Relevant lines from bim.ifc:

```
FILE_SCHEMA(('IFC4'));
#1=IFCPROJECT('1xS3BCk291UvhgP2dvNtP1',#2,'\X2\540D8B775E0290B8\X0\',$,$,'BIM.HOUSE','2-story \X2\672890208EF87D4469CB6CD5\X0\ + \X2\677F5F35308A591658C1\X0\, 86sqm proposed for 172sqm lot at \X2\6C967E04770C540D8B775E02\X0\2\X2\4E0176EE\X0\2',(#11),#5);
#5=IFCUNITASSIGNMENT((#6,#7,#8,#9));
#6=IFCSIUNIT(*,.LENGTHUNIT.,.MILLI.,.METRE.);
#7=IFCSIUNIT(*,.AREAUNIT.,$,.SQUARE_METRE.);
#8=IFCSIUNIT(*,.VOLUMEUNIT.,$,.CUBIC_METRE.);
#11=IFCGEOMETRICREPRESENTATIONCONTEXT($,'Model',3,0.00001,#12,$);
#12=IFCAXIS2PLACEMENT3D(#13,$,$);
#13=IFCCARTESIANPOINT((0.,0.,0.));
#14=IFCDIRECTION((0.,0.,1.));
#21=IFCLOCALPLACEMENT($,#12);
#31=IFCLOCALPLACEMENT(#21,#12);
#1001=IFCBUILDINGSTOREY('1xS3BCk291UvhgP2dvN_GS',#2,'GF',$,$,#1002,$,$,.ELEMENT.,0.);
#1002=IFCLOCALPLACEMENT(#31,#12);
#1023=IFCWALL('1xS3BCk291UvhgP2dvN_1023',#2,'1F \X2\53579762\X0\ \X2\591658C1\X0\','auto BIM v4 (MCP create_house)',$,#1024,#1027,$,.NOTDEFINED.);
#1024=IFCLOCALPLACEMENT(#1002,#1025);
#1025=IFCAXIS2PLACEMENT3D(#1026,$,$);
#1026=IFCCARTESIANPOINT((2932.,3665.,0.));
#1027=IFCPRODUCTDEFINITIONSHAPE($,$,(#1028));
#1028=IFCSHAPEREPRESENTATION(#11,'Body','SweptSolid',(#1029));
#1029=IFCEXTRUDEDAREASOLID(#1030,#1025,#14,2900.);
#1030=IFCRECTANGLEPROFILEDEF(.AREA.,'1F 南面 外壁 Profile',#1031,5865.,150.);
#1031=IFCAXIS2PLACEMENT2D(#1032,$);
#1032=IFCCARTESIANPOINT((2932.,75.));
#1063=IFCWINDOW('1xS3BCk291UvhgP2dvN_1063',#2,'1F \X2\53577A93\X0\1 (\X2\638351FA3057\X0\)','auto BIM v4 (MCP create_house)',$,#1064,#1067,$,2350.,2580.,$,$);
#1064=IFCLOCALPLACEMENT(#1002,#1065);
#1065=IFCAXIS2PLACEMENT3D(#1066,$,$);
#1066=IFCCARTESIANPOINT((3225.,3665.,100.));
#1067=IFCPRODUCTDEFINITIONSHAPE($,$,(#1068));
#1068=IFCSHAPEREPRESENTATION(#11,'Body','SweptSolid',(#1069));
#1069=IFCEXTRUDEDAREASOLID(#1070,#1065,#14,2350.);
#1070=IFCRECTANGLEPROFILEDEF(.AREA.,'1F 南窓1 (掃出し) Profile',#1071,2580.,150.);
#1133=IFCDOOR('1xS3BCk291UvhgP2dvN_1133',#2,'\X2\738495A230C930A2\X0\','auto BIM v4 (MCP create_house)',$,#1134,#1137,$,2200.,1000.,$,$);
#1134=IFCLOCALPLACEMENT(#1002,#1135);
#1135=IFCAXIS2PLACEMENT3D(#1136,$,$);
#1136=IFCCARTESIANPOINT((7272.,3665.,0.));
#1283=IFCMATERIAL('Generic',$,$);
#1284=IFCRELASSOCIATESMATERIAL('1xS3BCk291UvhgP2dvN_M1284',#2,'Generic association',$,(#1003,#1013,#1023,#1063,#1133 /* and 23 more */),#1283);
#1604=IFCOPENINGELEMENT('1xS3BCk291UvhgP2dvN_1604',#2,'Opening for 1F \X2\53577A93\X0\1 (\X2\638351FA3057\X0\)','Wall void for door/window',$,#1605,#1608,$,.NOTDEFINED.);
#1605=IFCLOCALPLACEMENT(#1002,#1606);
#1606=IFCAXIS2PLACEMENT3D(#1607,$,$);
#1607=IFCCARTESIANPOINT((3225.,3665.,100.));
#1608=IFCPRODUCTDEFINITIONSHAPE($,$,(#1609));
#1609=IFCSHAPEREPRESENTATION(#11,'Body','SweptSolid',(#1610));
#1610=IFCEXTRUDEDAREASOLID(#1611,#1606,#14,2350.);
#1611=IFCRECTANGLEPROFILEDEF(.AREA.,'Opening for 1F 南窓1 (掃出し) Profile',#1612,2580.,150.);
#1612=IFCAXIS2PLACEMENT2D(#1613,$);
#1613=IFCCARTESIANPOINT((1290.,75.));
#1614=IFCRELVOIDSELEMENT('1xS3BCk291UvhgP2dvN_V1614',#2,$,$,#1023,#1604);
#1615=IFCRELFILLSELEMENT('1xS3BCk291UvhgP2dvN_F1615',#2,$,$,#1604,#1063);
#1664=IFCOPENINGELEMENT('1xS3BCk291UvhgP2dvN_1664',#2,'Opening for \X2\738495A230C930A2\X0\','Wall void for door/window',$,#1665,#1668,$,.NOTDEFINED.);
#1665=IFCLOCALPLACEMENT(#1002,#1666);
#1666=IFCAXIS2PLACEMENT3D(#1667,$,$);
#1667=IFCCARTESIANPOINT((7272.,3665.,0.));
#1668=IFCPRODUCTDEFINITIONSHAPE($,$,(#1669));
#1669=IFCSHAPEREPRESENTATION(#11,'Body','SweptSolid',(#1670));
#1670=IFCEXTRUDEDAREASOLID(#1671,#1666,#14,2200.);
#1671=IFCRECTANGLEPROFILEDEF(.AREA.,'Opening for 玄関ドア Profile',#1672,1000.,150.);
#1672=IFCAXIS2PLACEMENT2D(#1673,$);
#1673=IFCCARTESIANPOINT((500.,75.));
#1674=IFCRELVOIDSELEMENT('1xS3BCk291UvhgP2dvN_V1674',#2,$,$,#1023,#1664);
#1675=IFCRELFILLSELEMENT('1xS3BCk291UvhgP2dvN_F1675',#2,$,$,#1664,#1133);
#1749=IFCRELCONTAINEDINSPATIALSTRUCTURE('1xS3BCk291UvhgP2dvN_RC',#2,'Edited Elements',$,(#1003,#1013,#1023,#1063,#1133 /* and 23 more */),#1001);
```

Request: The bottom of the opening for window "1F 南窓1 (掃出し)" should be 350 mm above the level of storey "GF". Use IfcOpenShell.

```python
import numpy as np
import ifcopenshell
import ifcopenshell.api.geometry
import ifcopenshell.geom
import ifcopenshell.util.element
import ifcopenshell.util.placement
import ifcopenshell.util.shape
import ifcopenshell.util.unit

model = ifcopenshell.open("bim.ifc")
unit_scale = ifcopenshell.util.unit.calculate_unit_scale(model)

window = model.by_guid("1xS3BCk291UvhgP2dvN_1063")
opening = window.FillsVoids[0].RelatingOpeningElement
storey = ifcopenshell.util.element.get_container(window, ifc_class="IfcBuildingStorey")
level = ifcopenshell.util.placement.get_local_placement(storey.ObjectPlacement)[2, 3]

# The opening's origin need not be at the sill, so measure its lowest point.
shape = ifcopenshell.geom.create_shape(ifcopenshell.geom.settings(), opening)
bottom = ifcopenshell.util.shape.get_shape_bottom_elevation(shape, shape.geometry) / unit_scale
dz = level + 0.35 / unit_scale - bottom

shift = np.array([0.0, 0.0, dz])
# The window is not placed relative to its opening, so move both.
for product in (opening, window):
    matrix = ifcopenshell.util.placement.get_local_placement(product.ObjectPlacement)
    matrix[:3, 3] += shift
    ifcopenshell.api.geometry.edit_object_placement(model, product=product, matrix=matrix, is_si=False)

print(f"moved by {dz * unit_scale:+.3f} m")

model.write("bim_updated.ifc")
```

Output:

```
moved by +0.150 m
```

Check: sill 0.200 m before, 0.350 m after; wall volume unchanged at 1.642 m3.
